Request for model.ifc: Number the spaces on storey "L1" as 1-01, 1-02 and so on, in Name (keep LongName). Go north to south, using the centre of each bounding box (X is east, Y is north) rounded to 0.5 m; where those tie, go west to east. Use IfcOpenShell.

First a look at what the model holds.

```python
import ifcopenshell
import ifcopenshell.util.element
import ifcopenshell.util.placement

model = ifcopenshell.open("model.ifc")
print(model.schema)
storey = next(s for s in model.by_type("IfcBuildingStorey") if s.Name == "L1")
spaces = [e for e in ifcopenshell.util.element.get_decomposition(storey) if e.is_a("IfcSpace")]
for e in sorted(spaces, key=lambda e: e.id()):
    origin = ifcopenshell.util.placement.get_local_placement(e.ObjectPlacement)[:3, 3]
    print(e.id(), e.Name, e.LongName, origin.round(2) + 0.0, sep=" | ")
```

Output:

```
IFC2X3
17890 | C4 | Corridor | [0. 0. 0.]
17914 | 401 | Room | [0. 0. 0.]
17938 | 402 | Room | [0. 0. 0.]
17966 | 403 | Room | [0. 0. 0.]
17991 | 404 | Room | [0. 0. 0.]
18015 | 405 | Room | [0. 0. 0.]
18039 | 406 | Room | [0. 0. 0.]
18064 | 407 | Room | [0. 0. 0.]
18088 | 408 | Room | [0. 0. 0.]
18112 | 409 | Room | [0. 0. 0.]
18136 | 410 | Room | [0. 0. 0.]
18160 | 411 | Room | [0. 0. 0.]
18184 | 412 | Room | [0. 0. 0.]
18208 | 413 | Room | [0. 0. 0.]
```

```python
import ifcopenshell
import ifcopenshell.geom
import ifcopenshell.util.element
import ifcopenshell.util.shape

model = ifcopenshell.open("model.ifc")
settings = ifcopenshell.geom.settings()
settings.set("use-world-coords", True)


def centre(element):
    shape = ifcopenshell.geom.create_shape(settings, element)
    return ifcopenshell.util.shape.get_bbox_centroid(shape.geometry)


storey = next(s for s in model.by_type("IfcBuildingStorey") if s.Name == "L1")
spaces = [e for e in ifcopenshell.util.element.get_decomposition(storey) if e.is_a("IfcSpace")]

# Insertion points can sit at a corner or the storey origin, so sort by the geometry (in metres).
centres = {e: centre(e) for e in spaces}
spaces.sort(key=lambda e: (-round(centres[e][1] / 0.5), centres[e][0]))

for i, e in enumerate(spaces, start=1):
    number = f"1-{i:02d}"
    e.Name = number
    print(e.id(), number)

model.write("model_v2.ifc")
```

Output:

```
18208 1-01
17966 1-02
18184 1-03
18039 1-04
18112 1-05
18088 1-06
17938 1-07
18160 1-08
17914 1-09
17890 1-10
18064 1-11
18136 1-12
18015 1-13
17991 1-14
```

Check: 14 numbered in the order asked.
